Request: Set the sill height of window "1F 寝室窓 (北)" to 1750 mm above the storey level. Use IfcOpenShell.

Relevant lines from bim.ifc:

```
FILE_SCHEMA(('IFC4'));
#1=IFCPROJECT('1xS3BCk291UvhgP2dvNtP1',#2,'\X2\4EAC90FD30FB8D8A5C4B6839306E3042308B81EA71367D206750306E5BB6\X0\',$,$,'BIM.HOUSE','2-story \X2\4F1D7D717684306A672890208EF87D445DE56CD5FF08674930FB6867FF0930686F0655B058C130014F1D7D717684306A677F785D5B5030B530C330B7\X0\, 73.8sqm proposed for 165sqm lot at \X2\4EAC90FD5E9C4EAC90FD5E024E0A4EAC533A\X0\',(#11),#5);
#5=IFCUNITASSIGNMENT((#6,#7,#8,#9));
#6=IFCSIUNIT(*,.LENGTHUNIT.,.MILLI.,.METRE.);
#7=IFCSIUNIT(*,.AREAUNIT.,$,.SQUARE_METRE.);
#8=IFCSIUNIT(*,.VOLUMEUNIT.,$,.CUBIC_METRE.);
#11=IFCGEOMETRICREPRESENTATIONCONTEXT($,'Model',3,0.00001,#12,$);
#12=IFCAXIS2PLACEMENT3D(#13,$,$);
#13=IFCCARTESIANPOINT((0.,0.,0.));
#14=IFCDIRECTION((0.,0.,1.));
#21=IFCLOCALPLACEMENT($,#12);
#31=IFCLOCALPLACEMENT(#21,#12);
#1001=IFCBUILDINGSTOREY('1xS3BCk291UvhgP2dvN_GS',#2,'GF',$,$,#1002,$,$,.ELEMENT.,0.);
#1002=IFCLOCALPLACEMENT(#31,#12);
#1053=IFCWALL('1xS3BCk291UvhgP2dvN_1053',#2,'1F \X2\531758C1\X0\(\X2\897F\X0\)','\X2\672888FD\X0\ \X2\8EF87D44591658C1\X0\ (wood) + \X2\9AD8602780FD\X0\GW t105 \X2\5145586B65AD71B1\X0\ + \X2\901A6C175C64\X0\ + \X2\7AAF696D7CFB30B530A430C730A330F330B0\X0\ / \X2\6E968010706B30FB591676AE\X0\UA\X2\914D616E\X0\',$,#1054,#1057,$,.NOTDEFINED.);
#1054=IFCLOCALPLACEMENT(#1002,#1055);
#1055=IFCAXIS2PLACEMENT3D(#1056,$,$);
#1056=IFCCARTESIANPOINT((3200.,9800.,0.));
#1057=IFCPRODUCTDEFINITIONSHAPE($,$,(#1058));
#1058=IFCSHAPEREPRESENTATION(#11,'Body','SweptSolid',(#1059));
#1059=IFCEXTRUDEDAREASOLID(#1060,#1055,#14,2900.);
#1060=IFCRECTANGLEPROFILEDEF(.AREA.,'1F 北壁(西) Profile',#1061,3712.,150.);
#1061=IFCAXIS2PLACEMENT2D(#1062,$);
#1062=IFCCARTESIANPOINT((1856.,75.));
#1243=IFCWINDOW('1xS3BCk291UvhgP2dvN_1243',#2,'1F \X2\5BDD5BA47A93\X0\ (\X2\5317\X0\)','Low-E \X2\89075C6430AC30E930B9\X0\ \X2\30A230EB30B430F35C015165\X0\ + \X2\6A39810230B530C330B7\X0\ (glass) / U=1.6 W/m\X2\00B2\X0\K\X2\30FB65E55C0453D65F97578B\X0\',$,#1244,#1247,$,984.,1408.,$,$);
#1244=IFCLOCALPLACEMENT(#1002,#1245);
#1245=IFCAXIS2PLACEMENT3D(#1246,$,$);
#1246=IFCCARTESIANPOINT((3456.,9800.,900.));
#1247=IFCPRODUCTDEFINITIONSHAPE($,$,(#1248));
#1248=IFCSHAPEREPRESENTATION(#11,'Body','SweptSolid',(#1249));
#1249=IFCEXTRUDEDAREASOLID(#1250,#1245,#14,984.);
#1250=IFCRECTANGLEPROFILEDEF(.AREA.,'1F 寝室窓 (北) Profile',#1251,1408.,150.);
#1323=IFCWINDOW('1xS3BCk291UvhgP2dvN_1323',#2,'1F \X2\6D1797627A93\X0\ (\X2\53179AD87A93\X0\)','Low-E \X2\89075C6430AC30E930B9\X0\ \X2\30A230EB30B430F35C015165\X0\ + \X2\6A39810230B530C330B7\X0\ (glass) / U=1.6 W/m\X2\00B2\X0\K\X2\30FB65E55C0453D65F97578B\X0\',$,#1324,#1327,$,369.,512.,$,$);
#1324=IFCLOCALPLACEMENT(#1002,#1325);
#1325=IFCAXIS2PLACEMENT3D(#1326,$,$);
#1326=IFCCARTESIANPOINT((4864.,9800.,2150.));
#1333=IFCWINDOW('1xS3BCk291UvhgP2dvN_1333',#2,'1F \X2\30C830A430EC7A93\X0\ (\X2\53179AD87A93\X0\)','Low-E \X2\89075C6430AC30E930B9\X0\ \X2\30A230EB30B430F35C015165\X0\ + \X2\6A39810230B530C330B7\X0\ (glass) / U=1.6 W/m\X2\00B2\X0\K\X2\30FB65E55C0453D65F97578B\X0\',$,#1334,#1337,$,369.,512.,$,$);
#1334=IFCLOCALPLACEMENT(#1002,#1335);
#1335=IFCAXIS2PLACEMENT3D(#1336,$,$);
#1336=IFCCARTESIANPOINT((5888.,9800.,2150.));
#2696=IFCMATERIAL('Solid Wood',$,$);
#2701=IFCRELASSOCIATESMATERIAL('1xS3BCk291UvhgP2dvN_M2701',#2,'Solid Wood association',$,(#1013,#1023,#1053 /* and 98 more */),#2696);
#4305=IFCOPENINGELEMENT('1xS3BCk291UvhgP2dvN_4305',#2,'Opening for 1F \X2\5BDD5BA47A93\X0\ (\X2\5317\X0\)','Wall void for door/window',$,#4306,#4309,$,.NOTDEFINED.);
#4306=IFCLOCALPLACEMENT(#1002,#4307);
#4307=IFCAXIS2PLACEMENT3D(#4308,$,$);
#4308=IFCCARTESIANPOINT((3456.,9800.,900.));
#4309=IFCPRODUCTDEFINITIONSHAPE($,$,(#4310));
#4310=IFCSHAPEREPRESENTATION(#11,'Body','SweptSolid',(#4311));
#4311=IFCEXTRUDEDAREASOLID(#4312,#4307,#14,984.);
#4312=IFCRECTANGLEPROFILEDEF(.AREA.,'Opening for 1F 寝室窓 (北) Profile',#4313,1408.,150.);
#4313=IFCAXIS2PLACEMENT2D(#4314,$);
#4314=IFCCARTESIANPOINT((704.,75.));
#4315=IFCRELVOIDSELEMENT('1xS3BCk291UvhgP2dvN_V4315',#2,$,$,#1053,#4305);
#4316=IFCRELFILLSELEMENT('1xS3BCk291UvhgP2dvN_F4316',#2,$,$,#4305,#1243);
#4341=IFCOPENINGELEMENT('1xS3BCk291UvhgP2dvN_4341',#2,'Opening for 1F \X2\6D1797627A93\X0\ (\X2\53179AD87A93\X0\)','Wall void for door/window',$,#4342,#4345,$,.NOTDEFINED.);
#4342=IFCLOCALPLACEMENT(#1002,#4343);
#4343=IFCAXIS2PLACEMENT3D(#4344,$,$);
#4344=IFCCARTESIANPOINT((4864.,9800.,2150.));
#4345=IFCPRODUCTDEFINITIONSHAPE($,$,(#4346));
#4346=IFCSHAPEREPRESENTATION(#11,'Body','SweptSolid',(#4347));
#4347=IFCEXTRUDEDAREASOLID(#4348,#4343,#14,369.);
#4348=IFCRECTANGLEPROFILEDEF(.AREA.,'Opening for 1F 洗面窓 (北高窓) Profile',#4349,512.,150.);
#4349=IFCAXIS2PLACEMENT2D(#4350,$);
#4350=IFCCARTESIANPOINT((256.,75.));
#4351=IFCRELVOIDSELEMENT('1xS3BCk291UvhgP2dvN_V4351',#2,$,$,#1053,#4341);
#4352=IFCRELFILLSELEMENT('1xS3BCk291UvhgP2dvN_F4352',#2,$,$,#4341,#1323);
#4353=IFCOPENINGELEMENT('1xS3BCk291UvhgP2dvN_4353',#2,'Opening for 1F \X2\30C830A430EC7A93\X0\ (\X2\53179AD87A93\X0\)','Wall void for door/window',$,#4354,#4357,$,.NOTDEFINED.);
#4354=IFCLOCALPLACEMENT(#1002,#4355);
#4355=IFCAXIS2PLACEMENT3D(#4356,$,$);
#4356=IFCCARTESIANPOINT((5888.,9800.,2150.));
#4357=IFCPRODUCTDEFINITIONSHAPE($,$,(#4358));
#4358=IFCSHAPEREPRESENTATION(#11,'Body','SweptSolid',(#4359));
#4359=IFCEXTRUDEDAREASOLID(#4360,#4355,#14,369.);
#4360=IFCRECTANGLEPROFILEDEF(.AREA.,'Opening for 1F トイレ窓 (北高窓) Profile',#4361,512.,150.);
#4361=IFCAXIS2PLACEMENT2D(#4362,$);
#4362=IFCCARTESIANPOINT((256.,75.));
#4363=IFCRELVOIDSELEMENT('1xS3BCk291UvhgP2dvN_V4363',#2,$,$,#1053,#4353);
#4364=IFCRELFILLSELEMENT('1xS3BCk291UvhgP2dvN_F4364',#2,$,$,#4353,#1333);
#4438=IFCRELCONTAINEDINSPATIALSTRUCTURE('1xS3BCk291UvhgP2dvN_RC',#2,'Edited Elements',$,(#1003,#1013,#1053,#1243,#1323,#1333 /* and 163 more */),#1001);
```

```python
import numpy as np
import ifcopenshell
import ifcopenshell.api.geometry
import ifcopenshell.geom
import ifcopenshell.util.element
import ifcopenshell.util.placement
import ifcopenshell.util.shape
import ifcopenshell.util.unit

model = ifcopenshell.open("bim.ifc")
unit_scale = ifcopenshell.util.unit.calculate_unit_scale(model)

window = model.by_guid("1xS3BCk291UvhgP2dvN_1243")
opening = window.FillsVoids[0].RelatingOpeningElement
storey = ifcopenshell.util.element.get_container(window, ifc_class="IfcBuildingStorey")
level = ifcopenshell.util.placement.get_local_placement(storey.ObjectPlacement)[2, 3]

# The opening's origin need not be at the sill, so measure its lowest point.
shape = ifcopenshell.geom.create_shape(ifcopenshell.geom.settings(), opening)
bottom = ifcopenshell.util.shape.get_shape_bottom_elevation(shape, shape.geometry) / unit_scale
dz = level + 1750.0 - bottom

shift = np.array([0.0, 0.0, dz])
# The window is not placed relative to its opening, so move both.
for product in (opening, window):
    matrix = ifcopenshell.util.placement.get_local_placement(product.ObjectPlacement)
    matrix[:3, 3] += shift
    ifcopenshell.api.geometry.edit_object_placement(model, product=product, matrix=matrix, is_si=False)

print(f"moved by {dz * unit_scale:+.3f} m")

model.write("bim-out.ifc")
```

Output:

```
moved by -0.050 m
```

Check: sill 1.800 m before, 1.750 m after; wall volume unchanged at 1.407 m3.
